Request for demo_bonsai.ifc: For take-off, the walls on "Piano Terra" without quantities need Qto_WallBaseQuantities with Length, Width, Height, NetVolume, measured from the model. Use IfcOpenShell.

First a look at what the model holds.

```python
import ifcopenshell
import ifcopenshell.util.element
import ifcopenshell.util.unit

model = ifcopenshell.open("demo_bonsai.ifc")
print(model.schema)
for unit_type in ("LENGTHUNIT", "AREAUNIT", "VOLUMEUNIT"):
    print(unit_type, ifcopenshell.util.unit.calculate_unit_scale(model, unit_type))
storey = next(s for s in model.by_type("IfcBuildingStorey") if s.Name == "Piano Terra")
walls = [e for e in ifcopenshell.util.element.get_decomposition(storey) if e.is_a("IfcWall")]
for e in sorted(walls, key=lambda e: e.id()):
    print(e.id(), e.is_a(), e.Name, list(ifcopenshell.util.element.get_psets(e, qtos_only=True)), sep=" | ")
```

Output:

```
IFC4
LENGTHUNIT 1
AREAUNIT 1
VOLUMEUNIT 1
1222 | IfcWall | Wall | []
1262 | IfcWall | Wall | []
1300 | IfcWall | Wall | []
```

```python
import ifcopenshell
import ifcopenshell.api.pset
import ifcopenshell.geom
import ifcopenshell.util.element
import ifcopenshell.util.shape
import ifcopenshell.util.unit

model = ifcopenshell.open("demo_bonsai.ifc")
unit_scale = ifcopenshell.util.unit.calculate_unit_scale(model)
volume_scale = ifcopenshell.util.unit.calculate_unit_scale(model, "VOLUMEUNIT")
settings = ifcopenshell.geom.settings()

storey = next(s for s in model.by_type("IfcBuildingStorey") if s.Name == "Piano Terra")
walls = [e for e in ifcopenshell.util.element.get_decomposition(storey) if e.is_a("IfcWall")]

for e in sorted(walls, key=lambda e: e.id()):
    if ifcopenshell.util.element.get_psets(e, qtos_only=True, should_inherit=False):
        continue
    # Geometry comes back in metres, in the element's own axes.
    shape = ifcopenshell.geom.create_shape(settings, e)
    values = {
        "Length": ifcopenshell.util.shape.get_x(shape.geometry) / unit_scale,
        "Width": ifcopenshell.util.shape.get_y(shape.geometry) / unit_scale,
        "Height": ifcopenshell.util.shape.get_z(shape.geometry) / unit_scale,
        "NetVolume": ifcopenshell.util.shape.get_volume(shape.geometry) / volume_scale,
    }
    qto = ifcopenshell.api.pset.add_qto(model, product=e, name="Qto_WallBaseQuantities")
    ifcopenshell.api.pset.edit_qto(model, qto=qto, properties=values)
    print(e.id(), {k: round(v, 3) for k, v in values.items()})

model.write("demo_bonsai_updated.ifc")
```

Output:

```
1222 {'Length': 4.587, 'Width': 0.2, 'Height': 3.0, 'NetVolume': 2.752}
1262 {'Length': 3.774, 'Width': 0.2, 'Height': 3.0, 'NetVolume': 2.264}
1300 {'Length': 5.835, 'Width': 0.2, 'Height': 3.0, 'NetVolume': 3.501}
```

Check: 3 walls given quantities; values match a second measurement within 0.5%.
